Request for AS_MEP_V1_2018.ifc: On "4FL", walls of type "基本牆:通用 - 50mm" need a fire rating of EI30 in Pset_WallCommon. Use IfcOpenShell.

First a look at what the model holds.

```python
import ifcopenshell
import ifcopenshell.util.element

model = ifcopenshell.open("AS_MEP_V1_2018.ifc")
print(model.schema)
storey = next(s for s in model.by_type("IfcBuildingStorey") if s.Name == "4FL")
walls = [e for e in ifcopenshell.util.element.get_decomposition(storey) if e.is_a("IfcWall")]
seen = {}
for e in walls:
    element_type = ifcopenshell.util.element.get_type(e)
    key = (element_type.Name if element_type != e and element_type else None, ifcopenshell.util.element.get_pset(e, "Pset_WallCommon", "FireRating"))
    seen[key] = seen.get(key, 0) + 1
for (name, value), count in sorted(seen.items(), key=str):
    print(count, "x", name, "|", value)
```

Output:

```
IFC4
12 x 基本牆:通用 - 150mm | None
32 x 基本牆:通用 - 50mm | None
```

```python
import ifcopenshell
import ifcopenshell.api.pset
import ifcopenshell.util.element

model = ifcopenshell.open("AS_MEP_V1_2018.ifc")

storey = next(s for s in model.by_type("IfcBuildingStorey") if s.Name == "4FL")
walls = [e for e in ifcopenshell.util.element.get_decomposition(storey) if e.is_a("IfcWall")]

count = 0
for e in walls:
    element_type = ifcopenshell.util.element.get_type(e)
    if element_type in (None, e) or element_type.Name != "基本牆:通用 - 50mm":
        continue
    # add_pset returns the element's existing set when there is one.
    pset = ifcopenshell.api.pset.add_pset(model, product=e, name="Pset_WallCommon")
    ifcopenshell.api.pset.edit_pset(model, pset=pset, properties={"FireRating": "EI30"})
    count += 1

print(count, "walls updated")

model.write("AS_MEP_V1_2018_updated.ifc")
```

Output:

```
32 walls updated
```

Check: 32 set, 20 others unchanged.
